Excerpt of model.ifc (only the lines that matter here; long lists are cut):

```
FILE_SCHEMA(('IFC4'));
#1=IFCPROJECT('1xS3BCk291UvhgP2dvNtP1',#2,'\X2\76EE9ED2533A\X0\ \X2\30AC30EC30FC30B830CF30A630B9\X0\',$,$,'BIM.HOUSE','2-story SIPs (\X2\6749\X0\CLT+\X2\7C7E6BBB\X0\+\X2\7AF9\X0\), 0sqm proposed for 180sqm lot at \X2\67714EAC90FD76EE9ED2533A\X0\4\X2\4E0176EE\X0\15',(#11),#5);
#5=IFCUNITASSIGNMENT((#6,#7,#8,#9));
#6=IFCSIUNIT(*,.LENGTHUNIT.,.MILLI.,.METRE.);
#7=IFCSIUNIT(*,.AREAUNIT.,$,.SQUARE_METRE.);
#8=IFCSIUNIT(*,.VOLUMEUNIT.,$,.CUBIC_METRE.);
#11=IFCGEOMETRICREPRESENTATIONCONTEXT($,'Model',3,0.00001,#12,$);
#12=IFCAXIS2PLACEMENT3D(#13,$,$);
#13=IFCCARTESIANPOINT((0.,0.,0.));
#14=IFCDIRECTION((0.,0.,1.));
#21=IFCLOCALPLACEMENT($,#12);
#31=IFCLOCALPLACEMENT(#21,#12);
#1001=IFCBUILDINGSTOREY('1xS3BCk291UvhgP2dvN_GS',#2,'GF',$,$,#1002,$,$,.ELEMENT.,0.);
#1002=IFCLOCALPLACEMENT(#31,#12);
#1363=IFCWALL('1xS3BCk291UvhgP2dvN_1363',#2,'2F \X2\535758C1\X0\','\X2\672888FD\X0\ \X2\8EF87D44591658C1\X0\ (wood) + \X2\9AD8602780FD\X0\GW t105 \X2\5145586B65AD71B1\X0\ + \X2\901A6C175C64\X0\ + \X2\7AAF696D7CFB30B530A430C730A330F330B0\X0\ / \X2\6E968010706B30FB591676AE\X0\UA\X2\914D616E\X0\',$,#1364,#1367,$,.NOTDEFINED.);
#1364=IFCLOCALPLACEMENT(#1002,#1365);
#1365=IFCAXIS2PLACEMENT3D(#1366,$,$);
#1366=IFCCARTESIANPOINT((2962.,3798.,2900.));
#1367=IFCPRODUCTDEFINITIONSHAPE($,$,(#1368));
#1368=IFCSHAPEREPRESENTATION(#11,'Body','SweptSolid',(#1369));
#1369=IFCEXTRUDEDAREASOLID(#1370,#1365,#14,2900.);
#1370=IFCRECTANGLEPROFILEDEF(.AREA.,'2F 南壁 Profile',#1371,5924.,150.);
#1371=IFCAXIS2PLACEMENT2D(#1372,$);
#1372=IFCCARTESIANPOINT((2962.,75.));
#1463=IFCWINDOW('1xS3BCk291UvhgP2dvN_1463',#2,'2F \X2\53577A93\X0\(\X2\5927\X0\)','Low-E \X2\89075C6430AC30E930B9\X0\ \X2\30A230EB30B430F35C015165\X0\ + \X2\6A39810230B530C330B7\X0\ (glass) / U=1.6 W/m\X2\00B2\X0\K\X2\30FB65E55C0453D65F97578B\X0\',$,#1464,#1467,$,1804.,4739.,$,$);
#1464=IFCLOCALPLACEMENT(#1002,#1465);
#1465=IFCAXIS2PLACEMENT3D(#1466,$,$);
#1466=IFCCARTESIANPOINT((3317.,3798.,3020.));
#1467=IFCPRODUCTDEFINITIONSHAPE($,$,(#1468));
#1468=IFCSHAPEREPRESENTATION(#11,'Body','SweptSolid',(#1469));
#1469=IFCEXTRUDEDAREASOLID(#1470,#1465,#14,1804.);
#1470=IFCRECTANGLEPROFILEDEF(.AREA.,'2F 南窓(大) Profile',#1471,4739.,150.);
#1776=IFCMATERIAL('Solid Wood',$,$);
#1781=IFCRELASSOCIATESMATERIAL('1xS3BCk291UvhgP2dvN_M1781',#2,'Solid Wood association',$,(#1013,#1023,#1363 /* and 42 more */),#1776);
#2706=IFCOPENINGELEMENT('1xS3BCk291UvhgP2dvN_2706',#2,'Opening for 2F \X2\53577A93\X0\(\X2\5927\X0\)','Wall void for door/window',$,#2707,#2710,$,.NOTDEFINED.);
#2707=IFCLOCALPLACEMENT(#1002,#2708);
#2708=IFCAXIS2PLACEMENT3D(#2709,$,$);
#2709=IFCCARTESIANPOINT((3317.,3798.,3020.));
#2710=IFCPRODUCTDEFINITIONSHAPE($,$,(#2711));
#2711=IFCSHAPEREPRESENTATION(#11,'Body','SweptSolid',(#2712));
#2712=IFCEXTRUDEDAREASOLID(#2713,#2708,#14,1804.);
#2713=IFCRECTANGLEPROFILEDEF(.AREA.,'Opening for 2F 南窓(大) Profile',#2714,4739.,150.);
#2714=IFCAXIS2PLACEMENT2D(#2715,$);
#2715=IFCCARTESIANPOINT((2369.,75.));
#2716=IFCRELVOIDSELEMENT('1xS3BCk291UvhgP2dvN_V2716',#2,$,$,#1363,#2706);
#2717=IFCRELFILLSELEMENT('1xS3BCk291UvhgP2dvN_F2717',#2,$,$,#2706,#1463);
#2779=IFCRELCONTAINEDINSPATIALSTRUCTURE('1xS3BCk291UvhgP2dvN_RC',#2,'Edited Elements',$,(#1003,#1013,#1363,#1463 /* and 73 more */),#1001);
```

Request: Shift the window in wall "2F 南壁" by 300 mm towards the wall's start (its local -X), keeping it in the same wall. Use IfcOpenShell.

```python
import ifcopenshell
import ifcopenshell.api.geometry
import ifcopenshell.util.placement

model = ifcopenshell.open("model.ifc")

window = model.by_guid("1xS3BCk291UvhgP2dvN_1463")
opening = window.FillsVoids[0].RelatingOpeningElement
wall = opening.VoidsElements[0].RelatingBuildingElement

wall_matrix = ifcopenshell.util.placement.get_local_placement(wall.ObjectPlacement)
shift = wall_matrix[:3, 0] * -300.0
before = ifcopenshell.util.placement.get_local_placement(window.ObjectPlacement)[:3, 3].copy()

# The window is not placed relative to its opening, so move both.
for product in (opening, window):
    matrix = ifcopenshell.util.placement.get_local_placement(product.ObjectPlacement)
    matrix[:3, 3] += shift
    ifcopenshell.api.geometry.edit_object_placement(model, product=product, matrix=matrix, is_si=False)

after = ifcopenshell.util.placement.get_local_placement(window.ObjectPlacement)[:3, 3]
print("window moved by", (after - before).round(3) + 0.0)

model.write("model_v2.ifc")
```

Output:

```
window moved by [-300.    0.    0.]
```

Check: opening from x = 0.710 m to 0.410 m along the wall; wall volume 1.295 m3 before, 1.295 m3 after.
